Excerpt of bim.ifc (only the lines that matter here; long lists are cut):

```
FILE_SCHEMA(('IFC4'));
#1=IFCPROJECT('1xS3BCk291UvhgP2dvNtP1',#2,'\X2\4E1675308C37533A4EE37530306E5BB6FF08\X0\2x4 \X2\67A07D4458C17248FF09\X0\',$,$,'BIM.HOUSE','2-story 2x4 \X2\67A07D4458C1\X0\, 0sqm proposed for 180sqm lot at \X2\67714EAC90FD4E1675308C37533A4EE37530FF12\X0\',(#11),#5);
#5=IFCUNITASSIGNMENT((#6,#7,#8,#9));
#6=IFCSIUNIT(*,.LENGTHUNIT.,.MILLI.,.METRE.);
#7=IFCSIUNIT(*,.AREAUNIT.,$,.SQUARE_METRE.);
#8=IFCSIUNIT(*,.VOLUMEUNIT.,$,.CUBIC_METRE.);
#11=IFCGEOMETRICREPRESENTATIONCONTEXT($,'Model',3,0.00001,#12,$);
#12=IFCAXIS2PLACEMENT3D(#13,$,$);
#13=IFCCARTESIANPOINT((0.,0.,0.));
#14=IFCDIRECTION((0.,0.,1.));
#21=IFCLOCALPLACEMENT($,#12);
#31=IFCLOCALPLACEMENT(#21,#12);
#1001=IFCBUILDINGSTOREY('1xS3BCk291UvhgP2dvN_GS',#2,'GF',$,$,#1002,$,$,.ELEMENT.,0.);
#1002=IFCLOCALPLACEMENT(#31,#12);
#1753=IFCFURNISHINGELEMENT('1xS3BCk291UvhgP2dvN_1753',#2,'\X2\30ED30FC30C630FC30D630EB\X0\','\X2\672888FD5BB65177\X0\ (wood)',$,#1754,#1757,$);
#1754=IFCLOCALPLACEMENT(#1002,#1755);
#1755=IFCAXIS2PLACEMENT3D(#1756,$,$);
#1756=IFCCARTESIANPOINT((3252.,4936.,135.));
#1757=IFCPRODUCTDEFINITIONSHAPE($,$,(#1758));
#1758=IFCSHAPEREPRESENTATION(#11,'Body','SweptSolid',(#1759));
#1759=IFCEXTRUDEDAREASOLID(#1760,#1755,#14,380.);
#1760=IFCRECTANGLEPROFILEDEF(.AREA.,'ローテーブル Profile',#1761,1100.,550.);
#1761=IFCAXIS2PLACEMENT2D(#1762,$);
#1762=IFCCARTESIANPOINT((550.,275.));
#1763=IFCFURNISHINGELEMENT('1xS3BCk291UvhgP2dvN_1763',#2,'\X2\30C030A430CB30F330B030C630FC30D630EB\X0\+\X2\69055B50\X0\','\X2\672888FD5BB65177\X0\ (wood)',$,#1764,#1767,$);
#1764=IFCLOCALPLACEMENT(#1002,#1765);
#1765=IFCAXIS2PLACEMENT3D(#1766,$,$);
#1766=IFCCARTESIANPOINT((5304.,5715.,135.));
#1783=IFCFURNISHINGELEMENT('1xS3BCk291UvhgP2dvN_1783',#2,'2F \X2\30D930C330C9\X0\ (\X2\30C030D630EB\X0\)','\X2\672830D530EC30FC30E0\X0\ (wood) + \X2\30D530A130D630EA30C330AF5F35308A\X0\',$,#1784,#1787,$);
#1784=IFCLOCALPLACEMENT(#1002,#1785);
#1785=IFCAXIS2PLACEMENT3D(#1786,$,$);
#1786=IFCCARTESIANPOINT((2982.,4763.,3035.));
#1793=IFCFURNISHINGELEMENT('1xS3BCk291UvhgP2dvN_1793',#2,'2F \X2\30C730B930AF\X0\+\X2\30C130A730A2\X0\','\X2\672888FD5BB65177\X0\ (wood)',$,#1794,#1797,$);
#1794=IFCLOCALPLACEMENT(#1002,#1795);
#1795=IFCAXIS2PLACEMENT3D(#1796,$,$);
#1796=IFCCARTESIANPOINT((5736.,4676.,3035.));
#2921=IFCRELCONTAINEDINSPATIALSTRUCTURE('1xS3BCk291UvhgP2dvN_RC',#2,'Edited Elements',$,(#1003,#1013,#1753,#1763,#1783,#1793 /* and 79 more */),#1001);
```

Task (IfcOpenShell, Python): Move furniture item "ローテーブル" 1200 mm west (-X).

```python
import ifcopenshell
import ifcopenshell.api.geometry
import ifcopenshell.util.placement

model = ifcopenshell.open("bim.ifc")

item = model.by_id(1753)
matrix = ifcopenshell.util.placement.get_local_placement(item.ObjectPlacement)
matrix[0, 3] -= 1200.0
ifcopenshell.api.geometry.edit_object_placement(model, product=item, matrix=matrix, is_si=False)

print(ifcopenshell.util.placement.get_local_placement(item.ObjectPlacement).round(3) + 0.0)

model.write("bim_v2.ifc")
```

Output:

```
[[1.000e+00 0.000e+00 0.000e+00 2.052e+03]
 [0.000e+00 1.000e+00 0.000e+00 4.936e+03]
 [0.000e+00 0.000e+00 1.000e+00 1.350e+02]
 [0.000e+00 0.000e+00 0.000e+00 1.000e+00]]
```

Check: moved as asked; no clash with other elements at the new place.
